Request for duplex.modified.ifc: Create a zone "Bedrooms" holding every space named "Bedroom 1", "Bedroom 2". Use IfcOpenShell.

First a look at what the model holds.

```python
import ifcopenshell

model = ifcopenshell.open("duplex.modified.ifc")
print(model.schema)
seen = {}
for space in model.by_type("IfcSpace"):
    seen[space.LongName] = seen.get(space.LongName, 0) + 1
for name, count in sorted(seen.items(), key=str):
    print(count, "x", name)
print("zones:", [z.Name for z in model.by_type("IfcZone")][:20])
```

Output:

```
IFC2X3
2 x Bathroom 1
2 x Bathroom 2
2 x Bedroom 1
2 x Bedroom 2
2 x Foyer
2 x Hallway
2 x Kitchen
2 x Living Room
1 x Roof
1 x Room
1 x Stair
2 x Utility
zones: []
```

```python
import ifcopenshell
import ifcopenshell.api.group
import ifcopenshell.api.root

model = ifcopenshell.open("duplex.modified.ifc")

names = {"Bedroom 1", "Bedroom 2"}
spaces = [s for s in model.by_type("IfcSpace") if s.LongName in names]

zone = ifcopenshell.api.root.create_entity(model, ifc_class="IfcZone", name="Bedrooms")
ifcopenshell.api.group.assign_group(model, products=spaces, group=zone)
print(len(spaces), "spaces in", zone.Name)

model.write("duplex.modified_updated.ifc")
```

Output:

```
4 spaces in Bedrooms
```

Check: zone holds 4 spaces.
